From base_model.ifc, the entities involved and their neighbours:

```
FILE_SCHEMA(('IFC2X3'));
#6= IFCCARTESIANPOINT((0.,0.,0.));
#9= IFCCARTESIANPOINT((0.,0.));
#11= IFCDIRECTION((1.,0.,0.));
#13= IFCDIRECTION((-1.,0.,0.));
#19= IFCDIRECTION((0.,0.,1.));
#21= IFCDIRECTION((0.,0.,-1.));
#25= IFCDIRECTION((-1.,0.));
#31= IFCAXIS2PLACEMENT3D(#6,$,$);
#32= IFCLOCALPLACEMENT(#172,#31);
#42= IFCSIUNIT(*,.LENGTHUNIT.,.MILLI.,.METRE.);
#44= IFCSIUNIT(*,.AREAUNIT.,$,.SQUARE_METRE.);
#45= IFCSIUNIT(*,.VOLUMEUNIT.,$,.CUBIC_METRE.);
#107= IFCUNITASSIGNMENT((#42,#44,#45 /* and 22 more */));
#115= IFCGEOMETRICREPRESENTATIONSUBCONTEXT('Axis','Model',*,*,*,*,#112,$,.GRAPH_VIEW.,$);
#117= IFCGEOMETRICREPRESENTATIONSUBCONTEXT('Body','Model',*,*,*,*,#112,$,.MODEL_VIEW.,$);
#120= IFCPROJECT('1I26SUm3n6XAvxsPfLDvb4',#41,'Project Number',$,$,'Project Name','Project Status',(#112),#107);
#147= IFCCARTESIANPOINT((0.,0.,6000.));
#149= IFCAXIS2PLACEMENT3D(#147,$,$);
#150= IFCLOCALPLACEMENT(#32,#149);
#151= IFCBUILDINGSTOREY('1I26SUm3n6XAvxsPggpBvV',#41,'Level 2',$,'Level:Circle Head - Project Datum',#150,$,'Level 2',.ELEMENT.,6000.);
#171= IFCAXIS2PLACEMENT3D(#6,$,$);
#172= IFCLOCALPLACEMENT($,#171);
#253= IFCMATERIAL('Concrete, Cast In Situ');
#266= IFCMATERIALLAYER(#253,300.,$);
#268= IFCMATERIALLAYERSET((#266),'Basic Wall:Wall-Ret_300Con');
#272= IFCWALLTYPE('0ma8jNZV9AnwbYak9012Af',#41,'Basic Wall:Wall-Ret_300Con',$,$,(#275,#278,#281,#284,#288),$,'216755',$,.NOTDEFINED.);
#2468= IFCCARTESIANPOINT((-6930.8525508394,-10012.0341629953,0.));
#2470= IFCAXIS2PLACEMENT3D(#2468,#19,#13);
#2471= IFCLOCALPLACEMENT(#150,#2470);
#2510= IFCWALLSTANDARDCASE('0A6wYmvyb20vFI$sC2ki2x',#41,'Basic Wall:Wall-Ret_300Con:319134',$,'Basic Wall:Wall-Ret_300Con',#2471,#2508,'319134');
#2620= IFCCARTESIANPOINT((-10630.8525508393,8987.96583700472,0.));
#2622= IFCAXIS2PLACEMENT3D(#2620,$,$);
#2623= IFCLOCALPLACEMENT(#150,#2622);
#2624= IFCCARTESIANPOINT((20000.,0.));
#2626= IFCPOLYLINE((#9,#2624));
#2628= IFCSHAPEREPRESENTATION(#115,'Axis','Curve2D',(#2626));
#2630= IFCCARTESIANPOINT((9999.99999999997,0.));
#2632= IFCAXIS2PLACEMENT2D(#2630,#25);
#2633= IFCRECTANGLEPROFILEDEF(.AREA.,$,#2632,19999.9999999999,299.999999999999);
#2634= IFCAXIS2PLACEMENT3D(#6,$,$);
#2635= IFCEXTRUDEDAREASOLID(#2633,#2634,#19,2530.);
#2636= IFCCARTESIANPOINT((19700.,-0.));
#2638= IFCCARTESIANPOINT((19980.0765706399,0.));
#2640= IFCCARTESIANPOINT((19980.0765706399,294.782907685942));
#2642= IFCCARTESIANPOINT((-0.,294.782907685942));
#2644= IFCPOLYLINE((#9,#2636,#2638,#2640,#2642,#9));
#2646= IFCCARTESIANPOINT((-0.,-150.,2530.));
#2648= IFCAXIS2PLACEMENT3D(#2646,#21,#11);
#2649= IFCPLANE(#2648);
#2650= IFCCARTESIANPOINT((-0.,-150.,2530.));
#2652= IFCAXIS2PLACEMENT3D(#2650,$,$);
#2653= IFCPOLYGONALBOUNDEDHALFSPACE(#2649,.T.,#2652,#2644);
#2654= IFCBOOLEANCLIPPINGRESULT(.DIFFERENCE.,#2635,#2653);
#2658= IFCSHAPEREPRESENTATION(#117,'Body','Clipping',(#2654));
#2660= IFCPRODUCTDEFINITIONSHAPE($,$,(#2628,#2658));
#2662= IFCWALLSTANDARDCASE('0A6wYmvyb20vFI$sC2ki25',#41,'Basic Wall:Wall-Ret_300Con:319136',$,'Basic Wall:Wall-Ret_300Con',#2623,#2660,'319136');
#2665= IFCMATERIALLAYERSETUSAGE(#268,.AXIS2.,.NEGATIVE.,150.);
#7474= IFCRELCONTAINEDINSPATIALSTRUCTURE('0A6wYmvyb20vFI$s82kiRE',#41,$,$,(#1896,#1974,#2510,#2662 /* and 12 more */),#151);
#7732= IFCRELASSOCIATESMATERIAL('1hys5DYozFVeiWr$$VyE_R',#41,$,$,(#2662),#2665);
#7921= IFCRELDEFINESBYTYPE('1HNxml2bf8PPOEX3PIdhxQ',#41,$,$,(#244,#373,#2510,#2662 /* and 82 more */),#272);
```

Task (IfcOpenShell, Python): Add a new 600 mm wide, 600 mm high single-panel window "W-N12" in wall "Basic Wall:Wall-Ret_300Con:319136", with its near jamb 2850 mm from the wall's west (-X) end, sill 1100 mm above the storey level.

```python
import numpy as np
import ifcopenshell
import ifcopenshell.api.feature
import ifcopenshell.api.geometry
import ifcopenshell.api.root
import ifcopenshell.api.spatial
import ifcopenshell.api.type
import ifcopenshell.geom
import ifcopenshell.util.element
import ifcopenshell.util.placement
import ifcopenshell.util.representation
import ifcopenshell.util.shape
import ifcopenshell.util.unit

model = ifcopenshell.open("base_model.ifc")
unit_scale = ifcopenshell.util.unit.calculate_unit_scale(model)
settings = ifcopenshell.geom.settings()


def volume(element):
    """Net volume in cubic metres, openings subtracted."""
    shape = ifcopenshell.geom.create_shape(settings, element)
    return ifcopenshell.util.shape.get_volume(shape.geometry)


wall = model.by_id(2662)
storey = ifcopenshell.util.element.get_container(wall, ifc_class="IfcBuildingStorey")
context = ifcopenshell.util.representation.get_context(model, "Model", "Body", "MODEL_VIEW")
before = volume(wall)

width, height, from_end, sill = 0.6, 0.6, 2.85, 1.1  # metres

# The wall runs along its own X axis, and the end named is its -X end.
wall_shape = ifcopenshell.geom.create_shape(settings, wall)
x, y, z = ifcopenshell.util.shape.get_vertices(wall_shape.geometry).T
start = x.min() + from_end
face, thickness = float(y.min()), float(y.max() - y.min())
wall_matrix = ifcopenshell.util.placement.get_local_placement(wall.ObjectPlacement)
level = ifcopenshell.util.placement.get_local_placement(storey.ObjectPlacement)[2, 3]


def in_wall(x, y):
    """Placement at x, y metres in the wall's axes, at sill height."""
    matrix = wall_matrix.copy()
    matrix[:, 3] = wall_matrix @ np.array([x / unit_scale, y / unit_scale, 0.0, 1.0])
    matrix[2, 3] = level + sill / unit_scale
    return matrix


# Opening: a box that overshoots both wall faces by 50 mm.
opening = ifcopenshell.api.root.create_entity(model, ifc_class="IfcOpeningElement")
box = ifcopenshell.api.geometry.add_wall_representation(
    model, context=context, length=width, height=height, thickness=thickness + 0.1
)
ifcopenshell.api.geometry.assign_representation(model, product=opening, representation=box)
ifcopenshell.api.geometry.edit_object_placement(model, product=opening, matrix=in_wall(start, face - 0.05), is_si=False)
ifcopenshell.api.feature.add_feature(model, feature=opening, element=wall)

window = ifcopenshell.api.root.create_entity(model, ifc_class="IfcWindow", name="W-N12")
window.OverallWidth, window.OverallHeight = width / unit_scale, height / unit_scale
body = ifcopenshell.api.geometry.add_window_representation(
    model,
    context=context,
    overall_width=window.OverallWidth,
    overall_height=window.OverallHeight,
    partition_type="SINGLE_PANEL",
)
ifcopenshell.api.geometry.assign_representation(model, product=window, representation=body)
ifcopenshell.api.spatial.assign_container(model, products=[window], relating_structure=storey)
fills = ifcopenshell.api.feature.add_filling(model, opening=opening, element=window)
fills.OwnerHistory = window.OwnerHistory  # required in IFC2X3

# IFC2X3 keeps the operation on the window style.
style = ifcopenshell.api.root.create_entity(model, ifc_class="IfcWindowStyle", name="W-N12")
style.OperationType, style.ConstructionType = "SINGLE_PANEL", "NOTDEFINED"
style.ParameterTakesPrecedence = style.Sizeable = False
ifcopenshell.api.type.assign_type(model, related_objects=[window], relating_type=style)

# Centre the window in the wall's thickness.
ifcopenshell.api.geometry.edit_object_placement(model, product=window, matrix=in_wall(start, face), is_si=False)
window_shape = ifcopenshell.geom.create_shape(settings, window)
depth = ifcopenshell.util.shape.get_vertices(window_shape.geometry)[:, 1]
offset = face + thickness / 2 - (depth.min() + depth.max()) / 2
ifcopenshell.api.geometry.edit_object_placement(model, product=window, matrix=in_wall(start, offset), is_si=False)

after = volume(wall)

print(f"wall volume {before:.3f} -> {after:.3f} m3")

model.write("base_model_rev.ifc")
```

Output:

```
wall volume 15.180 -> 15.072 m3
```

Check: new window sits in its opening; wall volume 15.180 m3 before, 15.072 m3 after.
